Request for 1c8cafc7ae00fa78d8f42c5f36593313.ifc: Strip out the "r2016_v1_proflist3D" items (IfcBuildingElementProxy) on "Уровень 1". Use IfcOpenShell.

First a look at what the model holds.

```python
import ifcopenshell
import ifcopenshell.util.element

model = ifcopenshell.open("1c8cafc7ae00fa78d8f42c5f36593313.ifc")
print(model.schema)
storey = next(s for s in model.by_type("IfcBuildingStorey") if s.Name == "Уровень 1")
proxies = [e for e in ifcopenshell.util.element.get_decomposition(storey) if e.is_a("IfcBuildingElementProxy")]
seen = {}
for e in proxies:
    element_type = ifcopenshell.util.element.get_type(e)
    name = element_type.Name if element_type not in (None, e) else None
    seen[name] = seen.get(name, 0) + 1
for name, count in sorted(seen.items(), key=str):
    print(count, "x", name)
```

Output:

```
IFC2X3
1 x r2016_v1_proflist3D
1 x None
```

```python
import ifcopenshell
import ifcopenshell.api.root
import ifcopenshell.util.element

model = ifcopenshell.open("1c8cafc7ae00fa78d8f42c5f36593313.ifc")

storey = next(s for s in model.by_type("IfcBuildingStorey") if s.Name == "Уровень 1")
proxies = [e for e in ifcopenshell.util.element.get_decomposition(storey) if e.is_a("IfcBuildingElementProxy")]
targets = [e for e in proxies if (t := ifcopenshell.util.element.get_type(e)) not in (None, e) and t.Name == "r2016_v1_proflist3D"]

for e in targets:
    ifcopenshell.api.root.remove_product(model, product=e)
print(len(targets), "removed")

model.write("1c8cafc7ae00fa78d8f42c5f36593313_v2.ifc")
```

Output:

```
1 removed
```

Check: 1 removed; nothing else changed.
